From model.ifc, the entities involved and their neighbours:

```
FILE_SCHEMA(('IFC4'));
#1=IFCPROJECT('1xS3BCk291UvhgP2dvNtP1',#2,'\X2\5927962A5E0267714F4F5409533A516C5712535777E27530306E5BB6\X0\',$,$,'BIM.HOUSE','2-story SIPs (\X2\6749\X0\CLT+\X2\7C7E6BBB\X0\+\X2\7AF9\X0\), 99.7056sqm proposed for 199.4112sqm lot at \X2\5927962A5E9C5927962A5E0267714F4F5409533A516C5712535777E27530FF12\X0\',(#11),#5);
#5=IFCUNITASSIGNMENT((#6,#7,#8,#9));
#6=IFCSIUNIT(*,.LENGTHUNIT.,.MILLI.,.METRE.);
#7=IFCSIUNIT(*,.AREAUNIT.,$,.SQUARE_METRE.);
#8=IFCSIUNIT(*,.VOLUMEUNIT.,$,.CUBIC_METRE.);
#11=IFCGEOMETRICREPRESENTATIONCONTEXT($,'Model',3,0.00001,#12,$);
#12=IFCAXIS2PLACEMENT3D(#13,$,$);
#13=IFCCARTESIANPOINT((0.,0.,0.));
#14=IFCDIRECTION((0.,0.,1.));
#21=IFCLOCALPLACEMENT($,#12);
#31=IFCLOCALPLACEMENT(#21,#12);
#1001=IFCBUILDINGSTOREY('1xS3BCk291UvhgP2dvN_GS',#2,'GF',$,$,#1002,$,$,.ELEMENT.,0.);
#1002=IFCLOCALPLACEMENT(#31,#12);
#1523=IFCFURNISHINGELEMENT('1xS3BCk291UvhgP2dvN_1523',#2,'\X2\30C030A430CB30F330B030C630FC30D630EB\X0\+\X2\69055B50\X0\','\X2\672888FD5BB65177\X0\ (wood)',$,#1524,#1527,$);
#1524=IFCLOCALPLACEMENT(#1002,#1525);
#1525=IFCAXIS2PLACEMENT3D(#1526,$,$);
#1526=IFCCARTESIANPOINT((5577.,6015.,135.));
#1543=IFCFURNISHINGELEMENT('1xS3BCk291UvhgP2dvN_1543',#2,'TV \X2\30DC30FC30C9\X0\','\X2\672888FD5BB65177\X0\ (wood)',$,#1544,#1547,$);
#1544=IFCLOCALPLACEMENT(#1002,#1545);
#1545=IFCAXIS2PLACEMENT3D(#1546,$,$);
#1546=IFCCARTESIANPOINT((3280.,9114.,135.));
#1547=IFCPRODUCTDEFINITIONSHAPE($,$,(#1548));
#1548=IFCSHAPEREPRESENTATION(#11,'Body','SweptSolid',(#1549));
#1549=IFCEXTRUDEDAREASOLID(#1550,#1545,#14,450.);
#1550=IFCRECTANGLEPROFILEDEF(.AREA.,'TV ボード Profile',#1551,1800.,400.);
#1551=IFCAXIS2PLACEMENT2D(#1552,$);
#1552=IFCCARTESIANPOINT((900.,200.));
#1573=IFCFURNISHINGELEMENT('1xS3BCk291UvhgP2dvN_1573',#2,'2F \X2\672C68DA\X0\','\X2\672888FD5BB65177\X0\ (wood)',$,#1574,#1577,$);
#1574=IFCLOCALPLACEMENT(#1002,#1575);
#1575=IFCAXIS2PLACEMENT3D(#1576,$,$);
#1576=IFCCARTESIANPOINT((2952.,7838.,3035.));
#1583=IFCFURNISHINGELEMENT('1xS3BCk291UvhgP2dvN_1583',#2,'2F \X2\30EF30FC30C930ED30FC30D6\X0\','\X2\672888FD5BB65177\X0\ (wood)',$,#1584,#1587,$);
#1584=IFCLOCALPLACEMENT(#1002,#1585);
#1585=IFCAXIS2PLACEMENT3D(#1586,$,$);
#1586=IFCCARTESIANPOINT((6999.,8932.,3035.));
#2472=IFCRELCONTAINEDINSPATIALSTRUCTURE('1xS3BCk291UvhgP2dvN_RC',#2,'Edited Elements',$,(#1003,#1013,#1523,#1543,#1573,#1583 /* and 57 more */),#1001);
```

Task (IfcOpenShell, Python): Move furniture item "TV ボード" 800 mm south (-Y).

```python
import ifcopenshell
import ifcopenshell.api.geometry
import ifcopenshell.util.placement

model = ifcopenshell.open("model.ifc")

item = model.by_id(1543)
matrix = ifcopenshell.util.placement.get_local_placement(item.ObjectPlacement)
matrix[1, 3] -= 800.0
ifcopenshell.api.geometry.edit_object_placement(model, product=item, matrix=matrix, is_si=False)

print(ifcopenshell.util.placement.get_local_placement(item.ObjectPlacement).round(3) + 0.0)

model.write("model_edited.ifc")
```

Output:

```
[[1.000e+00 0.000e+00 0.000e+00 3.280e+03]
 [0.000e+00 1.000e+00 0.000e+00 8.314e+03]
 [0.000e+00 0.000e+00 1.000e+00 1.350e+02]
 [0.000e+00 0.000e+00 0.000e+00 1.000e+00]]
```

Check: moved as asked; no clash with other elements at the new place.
